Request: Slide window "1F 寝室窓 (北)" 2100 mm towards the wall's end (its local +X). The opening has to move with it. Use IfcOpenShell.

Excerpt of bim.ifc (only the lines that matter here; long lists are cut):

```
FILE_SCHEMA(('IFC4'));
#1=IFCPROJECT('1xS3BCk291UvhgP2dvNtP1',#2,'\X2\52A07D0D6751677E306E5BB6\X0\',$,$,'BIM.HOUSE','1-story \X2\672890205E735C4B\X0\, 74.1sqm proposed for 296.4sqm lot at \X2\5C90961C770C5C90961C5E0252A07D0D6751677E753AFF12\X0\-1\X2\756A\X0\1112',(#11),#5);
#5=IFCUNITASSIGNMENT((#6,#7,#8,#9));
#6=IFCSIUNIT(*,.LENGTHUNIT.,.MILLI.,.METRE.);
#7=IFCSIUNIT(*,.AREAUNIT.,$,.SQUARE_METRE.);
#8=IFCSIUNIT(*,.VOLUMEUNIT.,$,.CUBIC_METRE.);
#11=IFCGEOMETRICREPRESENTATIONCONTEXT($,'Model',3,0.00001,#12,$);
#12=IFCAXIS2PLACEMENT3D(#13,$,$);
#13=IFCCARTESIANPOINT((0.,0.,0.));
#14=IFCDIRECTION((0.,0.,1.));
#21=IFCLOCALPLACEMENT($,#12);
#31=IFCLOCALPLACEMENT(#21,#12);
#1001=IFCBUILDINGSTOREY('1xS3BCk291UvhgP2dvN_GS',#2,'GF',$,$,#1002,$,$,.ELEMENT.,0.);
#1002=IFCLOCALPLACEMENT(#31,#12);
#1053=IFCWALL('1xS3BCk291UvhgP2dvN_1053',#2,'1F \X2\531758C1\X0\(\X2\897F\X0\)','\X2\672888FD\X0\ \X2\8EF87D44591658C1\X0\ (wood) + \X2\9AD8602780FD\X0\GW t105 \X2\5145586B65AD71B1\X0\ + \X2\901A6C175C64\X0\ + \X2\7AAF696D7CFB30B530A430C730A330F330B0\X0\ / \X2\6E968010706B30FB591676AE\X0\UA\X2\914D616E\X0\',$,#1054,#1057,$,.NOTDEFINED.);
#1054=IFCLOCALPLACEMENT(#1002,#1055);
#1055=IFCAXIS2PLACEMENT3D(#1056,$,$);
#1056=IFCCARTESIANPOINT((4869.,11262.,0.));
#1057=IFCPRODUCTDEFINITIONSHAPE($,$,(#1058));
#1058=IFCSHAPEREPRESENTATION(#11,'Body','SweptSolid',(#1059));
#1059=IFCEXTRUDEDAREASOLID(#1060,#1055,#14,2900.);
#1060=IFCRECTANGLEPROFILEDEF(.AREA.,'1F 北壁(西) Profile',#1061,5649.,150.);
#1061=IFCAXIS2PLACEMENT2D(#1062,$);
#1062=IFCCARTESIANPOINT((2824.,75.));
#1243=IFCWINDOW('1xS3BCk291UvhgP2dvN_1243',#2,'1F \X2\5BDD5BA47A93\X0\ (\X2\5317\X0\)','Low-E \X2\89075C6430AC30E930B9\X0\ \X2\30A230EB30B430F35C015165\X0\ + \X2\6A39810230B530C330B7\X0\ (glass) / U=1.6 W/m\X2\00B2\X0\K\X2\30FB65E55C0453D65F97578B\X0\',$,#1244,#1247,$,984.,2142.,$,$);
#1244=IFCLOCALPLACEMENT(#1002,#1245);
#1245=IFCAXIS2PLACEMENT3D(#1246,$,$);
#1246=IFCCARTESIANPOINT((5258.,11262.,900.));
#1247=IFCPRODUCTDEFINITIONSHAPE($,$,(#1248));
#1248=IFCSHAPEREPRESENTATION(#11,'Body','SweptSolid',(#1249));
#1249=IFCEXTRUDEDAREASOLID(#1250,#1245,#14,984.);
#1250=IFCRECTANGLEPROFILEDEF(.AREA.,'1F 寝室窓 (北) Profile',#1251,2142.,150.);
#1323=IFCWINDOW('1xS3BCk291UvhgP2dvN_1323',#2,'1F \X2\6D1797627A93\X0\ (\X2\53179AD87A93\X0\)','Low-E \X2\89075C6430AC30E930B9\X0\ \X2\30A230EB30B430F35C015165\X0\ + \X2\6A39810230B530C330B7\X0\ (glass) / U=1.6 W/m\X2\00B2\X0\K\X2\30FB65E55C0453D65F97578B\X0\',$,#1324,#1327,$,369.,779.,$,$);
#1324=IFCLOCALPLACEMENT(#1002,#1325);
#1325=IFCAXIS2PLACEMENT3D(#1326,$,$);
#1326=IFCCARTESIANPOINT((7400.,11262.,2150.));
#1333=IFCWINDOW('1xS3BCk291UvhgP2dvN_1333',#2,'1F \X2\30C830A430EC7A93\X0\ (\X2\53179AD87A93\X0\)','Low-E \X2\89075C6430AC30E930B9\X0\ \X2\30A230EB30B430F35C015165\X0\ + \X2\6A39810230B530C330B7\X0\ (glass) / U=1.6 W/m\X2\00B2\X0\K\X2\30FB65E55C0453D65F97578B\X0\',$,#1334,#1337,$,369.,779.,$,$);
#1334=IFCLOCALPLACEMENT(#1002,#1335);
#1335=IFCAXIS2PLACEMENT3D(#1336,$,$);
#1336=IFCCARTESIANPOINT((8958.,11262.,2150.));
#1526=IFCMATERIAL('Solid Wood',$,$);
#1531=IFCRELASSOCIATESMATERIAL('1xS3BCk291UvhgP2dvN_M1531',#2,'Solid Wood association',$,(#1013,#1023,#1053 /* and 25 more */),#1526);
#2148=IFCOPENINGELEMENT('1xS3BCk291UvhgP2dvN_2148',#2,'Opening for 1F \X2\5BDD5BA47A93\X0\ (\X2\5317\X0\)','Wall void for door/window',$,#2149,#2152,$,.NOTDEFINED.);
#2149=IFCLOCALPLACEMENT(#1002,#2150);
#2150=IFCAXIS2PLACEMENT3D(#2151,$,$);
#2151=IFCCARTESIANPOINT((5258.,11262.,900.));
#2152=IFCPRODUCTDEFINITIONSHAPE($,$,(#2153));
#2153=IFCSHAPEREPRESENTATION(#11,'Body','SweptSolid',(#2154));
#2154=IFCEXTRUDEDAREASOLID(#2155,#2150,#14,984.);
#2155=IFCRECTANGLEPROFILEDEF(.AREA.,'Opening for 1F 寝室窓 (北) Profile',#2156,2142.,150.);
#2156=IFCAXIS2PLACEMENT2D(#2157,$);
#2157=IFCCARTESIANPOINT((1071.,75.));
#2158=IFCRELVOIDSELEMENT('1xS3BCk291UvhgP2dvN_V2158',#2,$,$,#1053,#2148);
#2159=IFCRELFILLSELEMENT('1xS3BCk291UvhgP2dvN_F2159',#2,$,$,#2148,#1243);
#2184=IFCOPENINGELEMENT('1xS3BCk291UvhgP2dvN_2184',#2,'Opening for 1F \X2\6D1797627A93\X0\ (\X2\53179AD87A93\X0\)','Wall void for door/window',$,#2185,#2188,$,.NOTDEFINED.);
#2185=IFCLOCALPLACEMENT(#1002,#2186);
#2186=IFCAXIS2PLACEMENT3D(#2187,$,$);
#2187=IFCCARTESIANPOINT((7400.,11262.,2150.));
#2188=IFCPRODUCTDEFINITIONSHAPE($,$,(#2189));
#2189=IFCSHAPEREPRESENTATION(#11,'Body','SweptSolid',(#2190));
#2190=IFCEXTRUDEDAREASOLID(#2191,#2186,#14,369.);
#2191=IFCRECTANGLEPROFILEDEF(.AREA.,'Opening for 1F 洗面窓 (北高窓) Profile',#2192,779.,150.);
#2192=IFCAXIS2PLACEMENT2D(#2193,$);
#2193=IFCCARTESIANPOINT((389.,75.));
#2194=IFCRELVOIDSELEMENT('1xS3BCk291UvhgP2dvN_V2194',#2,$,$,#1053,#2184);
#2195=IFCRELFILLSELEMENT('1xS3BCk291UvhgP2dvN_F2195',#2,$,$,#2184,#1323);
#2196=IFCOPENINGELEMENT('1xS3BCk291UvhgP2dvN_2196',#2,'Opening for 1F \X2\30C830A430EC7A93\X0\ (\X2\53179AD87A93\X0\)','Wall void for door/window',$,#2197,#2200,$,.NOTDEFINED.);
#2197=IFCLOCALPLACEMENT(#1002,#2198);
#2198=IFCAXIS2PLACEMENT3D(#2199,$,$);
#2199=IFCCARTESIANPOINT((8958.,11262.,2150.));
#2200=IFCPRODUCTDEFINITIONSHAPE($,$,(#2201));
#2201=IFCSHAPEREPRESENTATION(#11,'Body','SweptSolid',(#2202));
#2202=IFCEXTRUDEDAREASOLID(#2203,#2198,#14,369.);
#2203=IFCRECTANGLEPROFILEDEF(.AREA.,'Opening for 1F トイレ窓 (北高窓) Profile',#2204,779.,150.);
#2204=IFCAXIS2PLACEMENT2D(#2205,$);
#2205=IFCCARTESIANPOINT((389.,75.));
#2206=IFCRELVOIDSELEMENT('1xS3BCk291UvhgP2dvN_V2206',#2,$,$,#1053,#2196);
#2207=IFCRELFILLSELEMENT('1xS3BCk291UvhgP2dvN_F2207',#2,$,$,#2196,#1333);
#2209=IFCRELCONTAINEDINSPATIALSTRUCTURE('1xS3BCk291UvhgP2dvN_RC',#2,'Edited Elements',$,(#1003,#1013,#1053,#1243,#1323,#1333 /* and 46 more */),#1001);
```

```python
import ifcopenshell
import ifcopenshell.api.geometry
import ifcopenshell.util.placement
import ifcopenshell.util.unit

model = ifcopenshell.open("bim.ifc")
unit_scale = ifcopenshell.util.unit.calculate_unit_scale(model)

window = model.by_guid("1xS3BCk291UvhgP2dvN_1243")
opening = window.FillsVoids[0].RelatingOpeningElement
wall = opening.VoidsElements[0].RelatingBuildingElement

wall_matrix = ifcopenshell.util.placement.get_local_placement(wall.ObjectPlacement)
shift = wall_matrix[:3, 0] * 2.1 / unit_scale
before = ifcopenshell.util.placement.get_local_placement(window.ObjectPlacement)[:3, 3].copy()

# The window is not placed relative to its opening, so move both.
for product in (opening, window):
    matrix = ifcopenshell.util.placement.get_local_placement(product.ObjectPlacement)
    matrix[:3, 3] += shift
    ifcopenshell.api.geometry.edit_object_placement(model, product=product, matrix=matrix, is_si=False)

after = ifcopenshell.util.placement.get_local_placement(window.ObjectPlacement)[:3, 3]
print("window moved by", (after - before).round(3) + 0.0)

model.write("bim_v2.ifc")
```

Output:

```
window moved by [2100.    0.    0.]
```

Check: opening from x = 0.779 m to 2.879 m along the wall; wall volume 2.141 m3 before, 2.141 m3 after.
